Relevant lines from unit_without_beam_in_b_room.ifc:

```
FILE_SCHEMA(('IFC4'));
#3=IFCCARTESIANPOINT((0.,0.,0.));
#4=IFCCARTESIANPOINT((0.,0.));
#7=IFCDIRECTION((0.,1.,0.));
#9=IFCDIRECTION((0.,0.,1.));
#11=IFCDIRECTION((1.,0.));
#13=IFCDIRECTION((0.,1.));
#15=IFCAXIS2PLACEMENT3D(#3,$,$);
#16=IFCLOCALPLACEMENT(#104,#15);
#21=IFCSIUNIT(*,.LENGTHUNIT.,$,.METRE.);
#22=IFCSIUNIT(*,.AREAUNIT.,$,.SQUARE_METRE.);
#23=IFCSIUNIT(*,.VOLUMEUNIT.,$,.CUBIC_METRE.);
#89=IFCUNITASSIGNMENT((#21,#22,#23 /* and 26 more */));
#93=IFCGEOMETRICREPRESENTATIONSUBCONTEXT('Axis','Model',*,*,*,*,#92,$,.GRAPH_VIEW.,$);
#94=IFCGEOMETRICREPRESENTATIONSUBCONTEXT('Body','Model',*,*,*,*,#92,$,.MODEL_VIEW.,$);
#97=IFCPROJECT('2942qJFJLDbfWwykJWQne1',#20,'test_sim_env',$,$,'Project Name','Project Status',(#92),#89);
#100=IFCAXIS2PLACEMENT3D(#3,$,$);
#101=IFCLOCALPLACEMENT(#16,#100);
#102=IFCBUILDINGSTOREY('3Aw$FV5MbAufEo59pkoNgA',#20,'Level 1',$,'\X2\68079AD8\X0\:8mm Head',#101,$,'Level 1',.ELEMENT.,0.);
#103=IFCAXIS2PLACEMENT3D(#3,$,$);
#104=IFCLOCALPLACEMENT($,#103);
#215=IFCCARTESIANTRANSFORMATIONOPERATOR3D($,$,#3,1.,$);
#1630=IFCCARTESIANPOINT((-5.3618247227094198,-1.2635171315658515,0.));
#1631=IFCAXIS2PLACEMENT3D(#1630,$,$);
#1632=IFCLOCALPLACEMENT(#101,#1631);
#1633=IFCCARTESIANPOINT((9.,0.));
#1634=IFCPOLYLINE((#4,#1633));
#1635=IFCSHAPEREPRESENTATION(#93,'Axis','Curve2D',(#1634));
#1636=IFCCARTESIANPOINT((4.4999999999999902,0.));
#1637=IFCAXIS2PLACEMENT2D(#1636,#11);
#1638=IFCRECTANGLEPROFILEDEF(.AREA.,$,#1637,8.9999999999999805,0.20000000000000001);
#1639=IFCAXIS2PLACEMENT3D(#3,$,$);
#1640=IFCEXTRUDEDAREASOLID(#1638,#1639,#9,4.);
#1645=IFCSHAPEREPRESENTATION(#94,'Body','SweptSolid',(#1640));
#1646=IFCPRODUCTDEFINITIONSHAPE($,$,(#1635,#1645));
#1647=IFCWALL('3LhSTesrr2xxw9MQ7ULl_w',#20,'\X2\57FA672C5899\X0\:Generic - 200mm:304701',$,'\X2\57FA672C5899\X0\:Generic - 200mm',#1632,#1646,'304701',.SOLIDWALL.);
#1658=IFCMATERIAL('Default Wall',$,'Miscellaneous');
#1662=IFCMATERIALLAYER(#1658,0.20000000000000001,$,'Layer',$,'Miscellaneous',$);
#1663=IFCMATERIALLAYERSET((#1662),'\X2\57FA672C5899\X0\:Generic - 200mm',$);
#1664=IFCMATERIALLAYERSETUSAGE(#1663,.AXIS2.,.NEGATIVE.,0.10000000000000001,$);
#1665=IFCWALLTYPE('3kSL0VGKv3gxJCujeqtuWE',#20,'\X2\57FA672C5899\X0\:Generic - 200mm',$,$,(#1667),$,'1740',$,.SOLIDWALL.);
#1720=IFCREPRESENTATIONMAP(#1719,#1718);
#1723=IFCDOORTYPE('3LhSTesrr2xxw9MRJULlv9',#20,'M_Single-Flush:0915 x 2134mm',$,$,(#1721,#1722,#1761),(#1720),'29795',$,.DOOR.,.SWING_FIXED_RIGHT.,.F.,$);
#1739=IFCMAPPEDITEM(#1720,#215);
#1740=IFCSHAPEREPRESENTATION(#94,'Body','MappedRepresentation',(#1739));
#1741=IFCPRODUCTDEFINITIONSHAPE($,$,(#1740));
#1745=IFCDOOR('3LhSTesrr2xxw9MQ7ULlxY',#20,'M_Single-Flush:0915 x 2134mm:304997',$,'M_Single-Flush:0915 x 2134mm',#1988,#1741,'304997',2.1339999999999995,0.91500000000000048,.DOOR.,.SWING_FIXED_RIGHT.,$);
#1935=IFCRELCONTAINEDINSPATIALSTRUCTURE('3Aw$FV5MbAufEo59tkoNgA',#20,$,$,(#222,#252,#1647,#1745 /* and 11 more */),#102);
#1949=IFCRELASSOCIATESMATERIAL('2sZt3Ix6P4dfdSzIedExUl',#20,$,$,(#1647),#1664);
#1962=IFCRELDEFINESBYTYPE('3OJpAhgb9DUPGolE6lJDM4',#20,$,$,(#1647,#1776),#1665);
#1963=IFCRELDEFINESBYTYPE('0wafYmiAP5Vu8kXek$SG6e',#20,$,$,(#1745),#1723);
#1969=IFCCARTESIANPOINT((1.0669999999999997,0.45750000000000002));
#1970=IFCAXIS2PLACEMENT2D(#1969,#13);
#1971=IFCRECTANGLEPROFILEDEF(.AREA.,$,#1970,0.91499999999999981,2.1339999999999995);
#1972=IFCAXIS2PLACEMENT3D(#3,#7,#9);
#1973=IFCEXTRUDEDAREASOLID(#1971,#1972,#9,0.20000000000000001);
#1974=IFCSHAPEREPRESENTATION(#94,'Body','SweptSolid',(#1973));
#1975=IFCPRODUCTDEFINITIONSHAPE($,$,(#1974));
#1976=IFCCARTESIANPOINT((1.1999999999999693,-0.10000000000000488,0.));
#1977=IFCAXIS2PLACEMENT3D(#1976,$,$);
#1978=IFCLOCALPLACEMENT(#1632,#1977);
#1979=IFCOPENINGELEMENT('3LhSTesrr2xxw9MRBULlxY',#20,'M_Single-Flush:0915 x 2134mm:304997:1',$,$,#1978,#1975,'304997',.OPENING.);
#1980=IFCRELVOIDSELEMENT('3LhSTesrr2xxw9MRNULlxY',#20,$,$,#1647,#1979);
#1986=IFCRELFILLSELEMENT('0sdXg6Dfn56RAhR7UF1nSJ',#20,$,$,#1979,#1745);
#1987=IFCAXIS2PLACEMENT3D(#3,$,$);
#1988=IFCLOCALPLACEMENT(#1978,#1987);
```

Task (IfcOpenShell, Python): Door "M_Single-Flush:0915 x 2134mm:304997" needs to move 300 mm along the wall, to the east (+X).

```python
import ifcopenshell
import ifcopenshell.api.geometry
import ifcopenshell.util.placement
import ifcopenshell.util.unit

model = ifcopenshell.open("unit_without_beam_in_b_room.ifc")
unit_scale = ifcopenshell.util.unit.calculate_unit_scale(model)

door = model.by_guid("3LhSTesrr2xxw9MQ7ULlxY")
opening = door.FillsVoids[0].RelatingOpeningElement
wall = opening.VoidsElements[0].RelatingBuildingElement

wall_matrix = ifcopenshell.util.placement.get_local_placement(wall.ObjectPlacement)
shift = wall_matrix[:3, 0] * 0.3 / unit_scale
before = ifcopenshell.util.placement.get_local_placement(door.ObjectPlacement)[:3, 3].copy()

# The door is placed relative to its opening, so it follows when the opening moves.
matrix = ifcopenshell.util.placement.get_local_placement(opening.ObjectPlacement)
matrix[:3, 3] += shift
ifcopenshell.api.geometry.edit_object_placement(
    model, product=opening, matrix=matrix, is_si=False, should_transform_children=True
)

after = ifcopenshell.util.placement.get_local_placement(door.ObjectPlacement)[:3, 3]
print("door moved by", (after - before).round(3) + 0.0)

model.write("unit_without_beam_in_b_room_v2.ifc")
```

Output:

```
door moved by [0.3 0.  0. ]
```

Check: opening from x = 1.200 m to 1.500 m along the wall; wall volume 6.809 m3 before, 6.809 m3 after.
